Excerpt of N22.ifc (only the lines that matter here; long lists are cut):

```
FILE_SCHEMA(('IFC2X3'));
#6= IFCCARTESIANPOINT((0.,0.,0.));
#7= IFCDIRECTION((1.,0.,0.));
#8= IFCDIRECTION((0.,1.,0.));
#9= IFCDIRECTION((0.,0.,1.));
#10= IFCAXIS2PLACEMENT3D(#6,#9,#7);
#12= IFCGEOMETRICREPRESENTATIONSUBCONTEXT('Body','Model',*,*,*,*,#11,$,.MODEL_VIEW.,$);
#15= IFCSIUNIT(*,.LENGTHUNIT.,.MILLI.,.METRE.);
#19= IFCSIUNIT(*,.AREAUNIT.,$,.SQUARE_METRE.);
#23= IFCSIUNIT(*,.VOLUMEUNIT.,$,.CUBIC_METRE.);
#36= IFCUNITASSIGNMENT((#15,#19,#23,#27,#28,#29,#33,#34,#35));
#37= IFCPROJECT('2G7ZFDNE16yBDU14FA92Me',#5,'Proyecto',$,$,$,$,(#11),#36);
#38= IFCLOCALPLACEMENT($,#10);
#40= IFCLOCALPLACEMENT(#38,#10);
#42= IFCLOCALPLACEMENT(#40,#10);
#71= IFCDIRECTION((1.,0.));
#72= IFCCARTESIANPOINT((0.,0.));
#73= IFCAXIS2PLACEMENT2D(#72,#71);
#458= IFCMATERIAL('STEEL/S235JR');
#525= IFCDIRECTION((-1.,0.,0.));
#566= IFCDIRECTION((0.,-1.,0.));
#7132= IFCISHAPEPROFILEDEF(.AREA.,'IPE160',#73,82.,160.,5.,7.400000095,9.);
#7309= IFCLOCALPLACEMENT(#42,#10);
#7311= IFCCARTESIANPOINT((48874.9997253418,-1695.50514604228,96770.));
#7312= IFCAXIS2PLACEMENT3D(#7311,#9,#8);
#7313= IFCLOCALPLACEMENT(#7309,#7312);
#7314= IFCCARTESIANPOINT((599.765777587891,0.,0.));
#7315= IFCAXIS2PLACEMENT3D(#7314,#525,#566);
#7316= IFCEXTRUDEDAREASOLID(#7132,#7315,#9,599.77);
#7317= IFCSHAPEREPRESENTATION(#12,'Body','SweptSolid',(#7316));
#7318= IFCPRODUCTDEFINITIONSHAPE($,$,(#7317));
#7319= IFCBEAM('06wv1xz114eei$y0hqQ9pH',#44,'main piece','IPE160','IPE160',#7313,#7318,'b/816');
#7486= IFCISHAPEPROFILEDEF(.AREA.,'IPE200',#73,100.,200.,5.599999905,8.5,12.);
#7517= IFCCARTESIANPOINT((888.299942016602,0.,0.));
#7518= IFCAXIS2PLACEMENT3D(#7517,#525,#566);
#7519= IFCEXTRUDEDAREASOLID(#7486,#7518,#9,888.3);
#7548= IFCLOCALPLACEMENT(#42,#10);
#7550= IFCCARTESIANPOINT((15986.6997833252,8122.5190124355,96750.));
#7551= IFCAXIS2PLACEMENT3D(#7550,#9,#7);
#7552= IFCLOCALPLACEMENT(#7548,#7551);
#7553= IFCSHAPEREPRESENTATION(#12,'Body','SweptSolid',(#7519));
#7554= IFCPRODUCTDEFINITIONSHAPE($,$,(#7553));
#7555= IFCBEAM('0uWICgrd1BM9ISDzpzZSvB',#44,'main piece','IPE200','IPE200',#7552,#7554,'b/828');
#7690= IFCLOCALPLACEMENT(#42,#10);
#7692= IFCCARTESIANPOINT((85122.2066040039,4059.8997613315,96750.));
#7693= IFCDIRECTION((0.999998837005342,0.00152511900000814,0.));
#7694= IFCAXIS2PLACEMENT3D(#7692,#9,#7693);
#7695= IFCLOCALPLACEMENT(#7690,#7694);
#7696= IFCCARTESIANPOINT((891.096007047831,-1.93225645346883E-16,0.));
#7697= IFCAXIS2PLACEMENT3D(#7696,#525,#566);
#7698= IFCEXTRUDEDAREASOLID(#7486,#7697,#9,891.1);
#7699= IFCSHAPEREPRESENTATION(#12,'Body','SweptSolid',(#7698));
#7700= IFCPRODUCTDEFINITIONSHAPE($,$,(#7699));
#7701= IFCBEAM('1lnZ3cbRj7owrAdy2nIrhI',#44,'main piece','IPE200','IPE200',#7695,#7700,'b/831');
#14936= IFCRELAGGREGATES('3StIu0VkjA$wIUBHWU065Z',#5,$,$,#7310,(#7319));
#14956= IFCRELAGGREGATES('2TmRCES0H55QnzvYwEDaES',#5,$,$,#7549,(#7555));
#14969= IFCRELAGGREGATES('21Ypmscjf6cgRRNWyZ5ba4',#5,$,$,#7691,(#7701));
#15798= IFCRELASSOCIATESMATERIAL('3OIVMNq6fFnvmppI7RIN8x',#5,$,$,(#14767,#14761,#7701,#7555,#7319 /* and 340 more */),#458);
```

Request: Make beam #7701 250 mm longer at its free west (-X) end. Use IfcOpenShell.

```python
import ifcopenshell
import ifcopenshell.util.representation
import ifcopenshell.util.unit

model = ifcopenshell.open("N22.ifc")
unit_scale = ifcopenshell.util.unit.calculate_unit_scale(model)

member = model.by_guid("1lnZ3cbRj7owrAdy2nIrhI")
change = 0.25 / unit_scale

# The extrusion runs towards the end named, so only its depth changes.
body = ifcopenshell.util.representation.get_representation(member, "Model", "Body")
solid = body.Items[0]
old_length = solid.Depth
solid.Depth += change

print(f"length {old_length:g} -> {solid.Depth:g}")

model.write("N22_edited.ifc")
```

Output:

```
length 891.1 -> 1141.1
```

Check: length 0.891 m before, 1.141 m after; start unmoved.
